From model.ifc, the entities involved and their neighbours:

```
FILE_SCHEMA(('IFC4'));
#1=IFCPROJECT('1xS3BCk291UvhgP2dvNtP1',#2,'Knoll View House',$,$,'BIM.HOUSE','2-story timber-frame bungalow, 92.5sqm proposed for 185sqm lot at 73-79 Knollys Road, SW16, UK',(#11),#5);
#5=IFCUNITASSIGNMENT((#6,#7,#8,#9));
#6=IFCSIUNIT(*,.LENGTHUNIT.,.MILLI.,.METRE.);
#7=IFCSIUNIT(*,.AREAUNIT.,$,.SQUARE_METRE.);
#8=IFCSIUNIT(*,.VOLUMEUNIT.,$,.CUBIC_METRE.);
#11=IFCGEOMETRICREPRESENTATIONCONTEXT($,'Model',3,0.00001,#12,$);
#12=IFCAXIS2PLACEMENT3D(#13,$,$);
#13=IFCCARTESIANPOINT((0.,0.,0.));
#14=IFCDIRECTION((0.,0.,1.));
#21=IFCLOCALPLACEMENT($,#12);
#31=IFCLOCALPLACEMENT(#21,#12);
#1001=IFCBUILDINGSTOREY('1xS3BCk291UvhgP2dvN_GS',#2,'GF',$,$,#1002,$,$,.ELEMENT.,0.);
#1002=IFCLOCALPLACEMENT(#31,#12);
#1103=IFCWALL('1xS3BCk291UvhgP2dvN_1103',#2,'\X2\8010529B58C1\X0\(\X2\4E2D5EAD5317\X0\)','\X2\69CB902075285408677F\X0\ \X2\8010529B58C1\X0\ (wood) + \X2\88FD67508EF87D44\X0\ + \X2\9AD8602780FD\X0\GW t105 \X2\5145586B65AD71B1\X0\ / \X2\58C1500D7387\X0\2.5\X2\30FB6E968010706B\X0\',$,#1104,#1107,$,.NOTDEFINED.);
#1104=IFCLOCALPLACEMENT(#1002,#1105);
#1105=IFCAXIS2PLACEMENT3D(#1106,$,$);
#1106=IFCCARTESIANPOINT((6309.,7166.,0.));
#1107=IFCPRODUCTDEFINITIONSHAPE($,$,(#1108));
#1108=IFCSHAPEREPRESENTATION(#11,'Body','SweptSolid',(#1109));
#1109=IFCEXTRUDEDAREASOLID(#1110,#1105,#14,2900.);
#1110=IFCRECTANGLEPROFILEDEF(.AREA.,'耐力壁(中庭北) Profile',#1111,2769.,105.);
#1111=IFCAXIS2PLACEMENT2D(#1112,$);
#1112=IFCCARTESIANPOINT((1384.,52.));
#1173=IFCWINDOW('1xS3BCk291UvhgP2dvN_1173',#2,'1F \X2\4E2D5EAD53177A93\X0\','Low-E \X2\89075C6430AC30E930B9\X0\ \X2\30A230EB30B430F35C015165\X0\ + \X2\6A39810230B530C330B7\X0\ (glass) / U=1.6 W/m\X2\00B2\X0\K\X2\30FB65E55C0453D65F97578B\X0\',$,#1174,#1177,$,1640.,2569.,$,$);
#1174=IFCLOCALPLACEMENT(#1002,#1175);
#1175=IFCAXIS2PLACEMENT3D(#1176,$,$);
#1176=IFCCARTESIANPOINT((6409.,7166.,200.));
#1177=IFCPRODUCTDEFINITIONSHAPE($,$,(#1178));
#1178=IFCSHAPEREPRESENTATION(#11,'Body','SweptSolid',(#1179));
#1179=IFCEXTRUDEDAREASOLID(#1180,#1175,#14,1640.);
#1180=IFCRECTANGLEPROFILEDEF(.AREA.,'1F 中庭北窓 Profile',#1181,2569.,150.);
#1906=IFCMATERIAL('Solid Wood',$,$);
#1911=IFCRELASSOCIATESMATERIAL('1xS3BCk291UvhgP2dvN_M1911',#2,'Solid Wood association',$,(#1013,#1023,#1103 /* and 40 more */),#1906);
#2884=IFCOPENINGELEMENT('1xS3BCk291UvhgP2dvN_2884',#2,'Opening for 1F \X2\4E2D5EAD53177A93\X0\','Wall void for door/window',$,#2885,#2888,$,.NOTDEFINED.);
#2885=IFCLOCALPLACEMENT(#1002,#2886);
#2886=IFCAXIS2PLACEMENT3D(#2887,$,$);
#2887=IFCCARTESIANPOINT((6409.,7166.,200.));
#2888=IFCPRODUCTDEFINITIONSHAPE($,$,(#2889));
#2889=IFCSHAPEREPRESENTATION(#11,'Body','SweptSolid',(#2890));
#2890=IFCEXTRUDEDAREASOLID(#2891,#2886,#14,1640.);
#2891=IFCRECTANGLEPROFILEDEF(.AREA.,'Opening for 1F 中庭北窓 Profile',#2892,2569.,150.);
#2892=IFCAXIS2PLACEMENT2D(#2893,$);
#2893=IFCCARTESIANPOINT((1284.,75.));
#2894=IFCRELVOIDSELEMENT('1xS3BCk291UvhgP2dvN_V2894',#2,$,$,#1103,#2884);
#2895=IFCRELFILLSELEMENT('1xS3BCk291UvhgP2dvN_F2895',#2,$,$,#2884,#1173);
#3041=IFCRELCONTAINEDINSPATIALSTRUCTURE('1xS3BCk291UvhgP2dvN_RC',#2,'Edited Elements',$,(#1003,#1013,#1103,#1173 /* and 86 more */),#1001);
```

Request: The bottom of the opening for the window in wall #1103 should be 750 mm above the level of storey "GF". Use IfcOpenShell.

```python
import numpy as np
import ifcopenshell
import ifcopenshell.api.geometry
import ifcopenshell.geom
import ifcopenshell.util.element
import ifcopenshell.util.placement
import ifcopenshell.util.shape
import ifcopenshell.util.unit

model = ifcopenshell.open("model.ifc")
unit_scale = ifcopenshell.util.unit.calculate_unit_scale(model)

window = model.by_id(1173)
opening = window.FillsVoids[0].RelatingOpeningElement
storey = ifcopenshell.util.element.get_container(window, ifc_class="IfcBuildingStorey")
level = ifcopenshell.util.placement.get_local_placement(storey.ObjectPlacement)[2, 3]

# The opening's origin need not be at the sill, so measure its lowest point.
shape = ifcopenshell.geom.create_shape(ifcopenshell.geom.settings(), opening)
bottom = ifcopenshell.util.shape.get_shape_bottom_elevation(shape, shape.geometry) / unit_scale
dz = level + 750.0 - bottom

shift = np.array([0.0, 0.0, dz])
# The window is not placed relative to its opening, so move both.
for product in (opening, window):
    matrix = ifcopenshell.util.placement.get_local_placement(product.ObjectPlacement)
    matrix[:3, 3] += shift
    ifcopenshell.api.geometry.edit_object_placement(model, product=product, matrix=matrix, is_si=False)

print(f"moved by {dz * unit_scale:+.3f} m")

model.write("model_edited.ifc")
```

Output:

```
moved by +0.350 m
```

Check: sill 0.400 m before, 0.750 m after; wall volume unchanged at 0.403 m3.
